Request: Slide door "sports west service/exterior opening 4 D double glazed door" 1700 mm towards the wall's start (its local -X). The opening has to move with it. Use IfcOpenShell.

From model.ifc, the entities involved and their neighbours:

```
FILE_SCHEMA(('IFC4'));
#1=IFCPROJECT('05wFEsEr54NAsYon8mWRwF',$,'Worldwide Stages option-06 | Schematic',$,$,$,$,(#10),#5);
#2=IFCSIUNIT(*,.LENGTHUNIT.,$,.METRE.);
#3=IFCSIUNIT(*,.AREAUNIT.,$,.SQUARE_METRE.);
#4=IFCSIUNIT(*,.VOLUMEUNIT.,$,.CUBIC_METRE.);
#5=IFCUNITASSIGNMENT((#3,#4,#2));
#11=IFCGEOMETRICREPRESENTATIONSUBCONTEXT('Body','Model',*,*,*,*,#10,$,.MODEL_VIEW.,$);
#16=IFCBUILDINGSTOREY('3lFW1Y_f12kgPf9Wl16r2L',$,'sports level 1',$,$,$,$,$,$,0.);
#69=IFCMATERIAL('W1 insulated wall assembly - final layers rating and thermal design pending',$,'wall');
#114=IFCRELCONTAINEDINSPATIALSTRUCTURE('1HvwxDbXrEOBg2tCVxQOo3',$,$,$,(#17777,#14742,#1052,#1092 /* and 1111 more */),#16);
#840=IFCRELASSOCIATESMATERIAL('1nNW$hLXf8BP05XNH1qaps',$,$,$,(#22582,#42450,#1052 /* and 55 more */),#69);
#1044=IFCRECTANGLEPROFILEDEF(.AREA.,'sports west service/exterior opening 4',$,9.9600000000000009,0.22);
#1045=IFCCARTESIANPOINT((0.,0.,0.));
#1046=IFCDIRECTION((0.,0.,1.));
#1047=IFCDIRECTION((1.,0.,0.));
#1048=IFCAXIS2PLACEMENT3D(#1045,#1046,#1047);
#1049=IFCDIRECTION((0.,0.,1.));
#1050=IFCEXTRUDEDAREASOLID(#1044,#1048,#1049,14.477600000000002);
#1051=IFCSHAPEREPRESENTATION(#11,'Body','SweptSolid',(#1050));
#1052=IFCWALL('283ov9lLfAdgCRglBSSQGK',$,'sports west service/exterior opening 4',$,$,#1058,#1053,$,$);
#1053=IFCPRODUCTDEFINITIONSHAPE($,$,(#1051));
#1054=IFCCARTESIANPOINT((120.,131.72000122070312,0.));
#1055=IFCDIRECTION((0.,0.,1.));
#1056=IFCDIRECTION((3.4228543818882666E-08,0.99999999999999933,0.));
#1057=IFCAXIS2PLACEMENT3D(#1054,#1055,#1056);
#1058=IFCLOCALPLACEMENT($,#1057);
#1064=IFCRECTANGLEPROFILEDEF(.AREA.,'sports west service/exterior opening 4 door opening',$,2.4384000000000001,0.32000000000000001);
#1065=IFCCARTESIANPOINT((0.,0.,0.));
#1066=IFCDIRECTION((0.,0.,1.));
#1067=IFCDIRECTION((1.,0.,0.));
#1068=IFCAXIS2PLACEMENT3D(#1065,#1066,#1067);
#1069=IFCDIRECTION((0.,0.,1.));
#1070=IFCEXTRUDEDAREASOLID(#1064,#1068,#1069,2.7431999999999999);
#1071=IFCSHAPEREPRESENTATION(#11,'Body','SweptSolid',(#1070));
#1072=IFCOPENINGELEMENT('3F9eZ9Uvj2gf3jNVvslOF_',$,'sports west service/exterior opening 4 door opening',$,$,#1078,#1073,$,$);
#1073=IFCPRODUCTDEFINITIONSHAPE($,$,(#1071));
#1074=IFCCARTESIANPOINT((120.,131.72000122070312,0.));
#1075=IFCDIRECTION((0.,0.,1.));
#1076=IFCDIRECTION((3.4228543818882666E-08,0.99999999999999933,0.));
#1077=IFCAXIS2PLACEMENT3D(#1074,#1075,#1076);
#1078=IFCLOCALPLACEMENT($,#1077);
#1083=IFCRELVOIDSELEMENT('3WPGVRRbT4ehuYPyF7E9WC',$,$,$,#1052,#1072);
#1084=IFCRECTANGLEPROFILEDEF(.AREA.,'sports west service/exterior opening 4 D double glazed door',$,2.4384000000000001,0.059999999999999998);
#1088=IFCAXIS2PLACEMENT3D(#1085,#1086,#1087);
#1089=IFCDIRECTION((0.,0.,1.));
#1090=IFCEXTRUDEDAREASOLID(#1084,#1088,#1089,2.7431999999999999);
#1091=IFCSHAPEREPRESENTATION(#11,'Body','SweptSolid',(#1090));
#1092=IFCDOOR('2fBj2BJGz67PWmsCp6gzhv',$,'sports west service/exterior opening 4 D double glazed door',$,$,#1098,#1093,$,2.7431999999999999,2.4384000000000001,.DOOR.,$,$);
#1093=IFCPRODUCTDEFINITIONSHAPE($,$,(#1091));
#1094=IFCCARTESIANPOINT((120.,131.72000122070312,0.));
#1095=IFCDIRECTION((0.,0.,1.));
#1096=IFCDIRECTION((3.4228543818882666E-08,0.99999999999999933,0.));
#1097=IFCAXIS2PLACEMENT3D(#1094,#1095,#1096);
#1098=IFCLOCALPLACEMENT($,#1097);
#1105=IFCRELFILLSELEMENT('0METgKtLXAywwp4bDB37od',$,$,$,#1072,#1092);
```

```python
import ifcopenshell
import ifcopenshell.api.geometry
import ifcopenshell.util.placement
import ifcopenshell.util.unit

model = ifcopenshell.open("model.ifc")
unit_scale = ifcopenshell.util.unit.calculate_unit_scale(model)

door = model.by_id(1092)
opening = door.FillsVoids[0].RelatingOpeningElement
wall = opening.VoidsElements[0].RelatingBuildingElement

wall_matrix = ifcopenshell.util.placement.get_local_placement(wall.ObjectPlacement)
shift = wall_matrix[:3, 0] * -1.7 / unit_scale
before = ifcopenshell.util.placement.get_local_placement(door.ObjectPlacement)[:3, 3].copy()

# The door is not placed relative to its opening, so move both.
for product in (opening, door):
    matrix = ifcopenshell.util.placement.get_local_placement(product.ObjectPlacement)
    matrix[:3, 3] += shift
    ifcopenshell.api.geometry.edit_object_placement(model, product=product, matrix=matrix, is_si=False)

after = ifcopenshell.util.placement.get_local_placement(door.ObjectPlacement)[:3, 3]
print("door moved by", (after - before).round(3) + 0.0)

model.write("model_v2.ifc")
```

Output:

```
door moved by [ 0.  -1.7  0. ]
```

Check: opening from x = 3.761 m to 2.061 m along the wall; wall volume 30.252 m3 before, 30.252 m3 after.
